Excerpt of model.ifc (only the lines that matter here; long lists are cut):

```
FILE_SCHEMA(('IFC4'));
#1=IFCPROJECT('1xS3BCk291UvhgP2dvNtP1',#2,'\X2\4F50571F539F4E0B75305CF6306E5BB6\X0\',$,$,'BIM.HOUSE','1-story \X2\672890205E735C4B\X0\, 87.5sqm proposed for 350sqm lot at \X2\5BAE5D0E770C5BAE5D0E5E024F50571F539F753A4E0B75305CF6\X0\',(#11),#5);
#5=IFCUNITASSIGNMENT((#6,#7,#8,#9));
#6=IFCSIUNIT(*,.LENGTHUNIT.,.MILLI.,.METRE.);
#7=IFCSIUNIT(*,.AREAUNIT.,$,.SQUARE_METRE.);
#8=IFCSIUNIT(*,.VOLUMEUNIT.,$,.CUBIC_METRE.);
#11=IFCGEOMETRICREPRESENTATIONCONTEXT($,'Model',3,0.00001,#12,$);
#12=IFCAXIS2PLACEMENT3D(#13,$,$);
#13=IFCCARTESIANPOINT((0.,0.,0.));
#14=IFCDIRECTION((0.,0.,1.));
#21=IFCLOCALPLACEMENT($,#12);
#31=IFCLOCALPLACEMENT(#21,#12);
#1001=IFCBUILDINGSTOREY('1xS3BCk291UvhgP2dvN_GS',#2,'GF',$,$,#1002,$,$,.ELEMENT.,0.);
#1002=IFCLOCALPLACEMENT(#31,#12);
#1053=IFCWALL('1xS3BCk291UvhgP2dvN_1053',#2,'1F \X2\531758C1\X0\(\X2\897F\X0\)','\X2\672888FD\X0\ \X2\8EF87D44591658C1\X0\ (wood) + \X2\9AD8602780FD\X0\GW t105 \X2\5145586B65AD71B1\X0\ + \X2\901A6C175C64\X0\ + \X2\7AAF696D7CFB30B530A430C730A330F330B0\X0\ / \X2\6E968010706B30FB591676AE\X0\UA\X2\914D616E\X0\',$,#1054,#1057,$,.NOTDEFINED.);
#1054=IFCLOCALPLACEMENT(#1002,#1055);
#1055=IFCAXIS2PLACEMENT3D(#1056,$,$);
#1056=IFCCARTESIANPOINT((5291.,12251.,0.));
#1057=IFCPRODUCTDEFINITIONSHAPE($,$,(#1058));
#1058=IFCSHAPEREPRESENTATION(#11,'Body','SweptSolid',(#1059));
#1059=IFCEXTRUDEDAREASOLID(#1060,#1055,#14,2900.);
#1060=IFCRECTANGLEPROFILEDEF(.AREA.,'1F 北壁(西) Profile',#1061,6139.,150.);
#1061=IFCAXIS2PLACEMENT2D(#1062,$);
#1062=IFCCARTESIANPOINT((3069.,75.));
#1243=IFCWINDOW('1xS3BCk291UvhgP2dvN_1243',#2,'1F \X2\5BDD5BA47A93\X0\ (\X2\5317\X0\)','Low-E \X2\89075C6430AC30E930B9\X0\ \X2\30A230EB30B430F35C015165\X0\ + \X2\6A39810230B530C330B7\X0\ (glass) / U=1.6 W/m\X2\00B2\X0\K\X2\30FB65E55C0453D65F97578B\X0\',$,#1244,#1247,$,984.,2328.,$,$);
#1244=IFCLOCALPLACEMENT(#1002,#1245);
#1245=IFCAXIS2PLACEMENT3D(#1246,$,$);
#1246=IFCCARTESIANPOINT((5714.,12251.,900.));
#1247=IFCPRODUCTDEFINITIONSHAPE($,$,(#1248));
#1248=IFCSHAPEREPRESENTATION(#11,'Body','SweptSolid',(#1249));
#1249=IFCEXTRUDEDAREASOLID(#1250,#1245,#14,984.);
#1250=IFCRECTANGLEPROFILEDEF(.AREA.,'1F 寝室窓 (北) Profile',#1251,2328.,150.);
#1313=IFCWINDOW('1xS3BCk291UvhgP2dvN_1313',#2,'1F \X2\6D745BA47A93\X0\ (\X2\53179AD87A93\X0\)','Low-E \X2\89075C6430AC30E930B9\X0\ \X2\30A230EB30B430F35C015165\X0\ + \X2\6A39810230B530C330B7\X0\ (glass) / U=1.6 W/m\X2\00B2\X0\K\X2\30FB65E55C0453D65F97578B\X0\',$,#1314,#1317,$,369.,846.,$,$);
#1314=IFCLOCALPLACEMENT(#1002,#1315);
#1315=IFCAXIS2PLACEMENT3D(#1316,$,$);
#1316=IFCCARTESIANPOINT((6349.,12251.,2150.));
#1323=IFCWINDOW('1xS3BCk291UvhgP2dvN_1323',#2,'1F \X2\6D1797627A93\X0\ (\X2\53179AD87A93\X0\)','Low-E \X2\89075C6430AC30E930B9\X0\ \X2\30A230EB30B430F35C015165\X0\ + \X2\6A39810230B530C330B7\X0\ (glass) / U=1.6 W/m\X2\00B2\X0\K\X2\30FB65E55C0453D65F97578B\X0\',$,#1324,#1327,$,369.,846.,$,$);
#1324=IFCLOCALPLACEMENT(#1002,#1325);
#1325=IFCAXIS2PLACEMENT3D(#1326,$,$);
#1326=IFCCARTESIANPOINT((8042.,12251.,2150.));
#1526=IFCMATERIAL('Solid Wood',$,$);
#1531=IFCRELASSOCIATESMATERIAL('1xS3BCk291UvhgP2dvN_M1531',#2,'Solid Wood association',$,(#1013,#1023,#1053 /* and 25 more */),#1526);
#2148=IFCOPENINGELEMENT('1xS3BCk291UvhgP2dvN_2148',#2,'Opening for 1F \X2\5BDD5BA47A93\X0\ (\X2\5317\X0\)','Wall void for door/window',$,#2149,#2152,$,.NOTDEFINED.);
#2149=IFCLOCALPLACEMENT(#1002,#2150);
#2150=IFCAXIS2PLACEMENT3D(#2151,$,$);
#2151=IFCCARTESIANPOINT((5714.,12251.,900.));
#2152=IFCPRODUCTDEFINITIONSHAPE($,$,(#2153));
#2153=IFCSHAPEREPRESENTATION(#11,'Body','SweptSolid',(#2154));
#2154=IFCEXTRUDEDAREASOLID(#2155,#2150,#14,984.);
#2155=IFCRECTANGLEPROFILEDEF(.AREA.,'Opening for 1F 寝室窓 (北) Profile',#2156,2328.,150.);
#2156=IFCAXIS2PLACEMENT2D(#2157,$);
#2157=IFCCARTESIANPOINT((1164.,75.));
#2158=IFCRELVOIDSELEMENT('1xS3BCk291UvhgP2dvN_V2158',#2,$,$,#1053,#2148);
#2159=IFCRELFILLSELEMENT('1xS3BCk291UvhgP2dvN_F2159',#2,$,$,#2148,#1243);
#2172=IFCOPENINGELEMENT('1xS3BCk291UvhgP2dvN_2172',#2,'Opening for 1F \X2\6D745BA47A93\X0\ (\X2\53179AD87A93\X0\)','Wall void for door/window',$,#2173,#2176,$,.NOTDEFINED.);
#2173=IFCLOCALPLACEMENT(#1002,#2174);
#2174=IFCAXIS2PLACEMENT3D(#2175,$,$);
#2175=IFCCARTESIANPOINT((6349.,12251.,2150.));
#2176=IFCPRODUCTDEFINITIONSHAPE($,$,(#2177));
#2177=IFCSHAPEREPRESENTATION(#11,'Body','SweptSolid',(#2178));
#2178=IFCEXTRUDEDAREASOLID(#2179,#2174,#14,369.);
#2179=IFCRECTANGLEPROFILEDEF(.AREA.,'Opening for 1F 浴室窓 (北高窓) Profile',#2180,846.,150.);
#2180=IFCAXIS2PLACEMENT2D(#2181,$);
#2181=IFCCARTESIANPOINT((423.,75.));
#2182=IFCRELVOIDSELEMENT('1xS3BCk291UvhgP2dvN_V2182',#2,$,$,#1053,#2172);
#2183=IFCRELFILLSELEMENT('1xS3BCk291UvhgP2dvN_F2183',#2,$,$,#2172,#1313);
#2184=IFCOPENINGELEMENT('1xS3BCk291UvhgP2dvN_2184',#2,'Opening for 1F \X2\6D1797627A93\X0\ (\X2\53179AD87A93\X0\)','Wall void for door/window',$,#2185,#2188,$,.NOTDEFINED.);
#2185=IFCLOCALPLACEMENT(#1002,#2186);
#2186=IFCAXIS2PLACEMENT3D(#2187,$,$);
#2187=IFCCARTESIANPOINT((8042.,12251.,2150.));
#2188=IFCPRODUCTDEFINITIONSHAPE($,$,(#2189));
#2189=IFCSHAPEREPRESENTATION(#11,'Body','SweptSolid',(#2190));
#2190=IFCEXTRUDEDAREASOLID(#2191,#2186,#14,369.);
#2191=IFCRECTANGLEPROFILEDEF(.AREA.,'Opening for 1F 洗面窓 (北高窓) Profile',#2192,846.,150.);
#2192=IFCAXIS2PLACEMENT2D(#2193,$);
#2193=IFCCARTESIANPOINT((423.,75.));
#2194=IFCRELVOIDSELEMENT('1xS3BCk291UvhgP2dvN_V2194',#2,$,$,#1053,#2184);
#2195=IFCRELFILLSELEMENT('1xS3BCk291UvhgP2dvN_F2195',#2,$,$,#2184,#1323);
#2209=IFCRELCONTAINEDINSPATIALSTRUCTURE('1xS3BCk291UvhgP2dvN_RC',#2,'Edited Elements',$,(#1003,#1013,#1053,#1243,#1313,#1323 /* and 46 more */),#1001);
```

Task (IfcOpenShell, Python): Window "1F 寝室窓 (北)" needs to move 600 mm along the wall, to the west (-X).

```python
import ifcopenshell
import ifcopenshell.api.geometry
import ifcopenshell.util.placement
import ifcopenshell.util.unit

model = ifcopenshell.open("model.ifc")
unit_scale = ifcopenshell.util.unit.calculate_unit_scale(model)

window = model.by_guid("1xS3BCk291UvhgP2dvN_1243")
opening = window.FillsVoids[0].RelatingOpeningElement
wall = opening.VoidsElements[0].RelatingBuildingElement

wall_matrix = ifcopenshell.util.placement.get_local_placement(wall.ObjectPlacement)
shift = wall_matrix[:3, 0] * -0.6 / unit_scale
before = ifcopenshell.util.placement.get_local_placement(window.ObjectPlacement)[:3, 3].copy()

# The window is not placed relative to its opening, so move both.
for product in (opening, window):
    matrix = ifcopenshell.util.placement.get_local_placement(product.ObjectPlacement)
    matrix[:3, 3] += shift
    ifcopenshell.api.geometry.edit_object_placement(model, product=product, matrix=matrix, is_si=False)

after = ifcopenshell.util.placement.get_local_placement(window.ObjectPlacement)[:3, 3]
print("window moved by", (after - before).round(3) + 0.0)

model.write("model_rev.ifc")
```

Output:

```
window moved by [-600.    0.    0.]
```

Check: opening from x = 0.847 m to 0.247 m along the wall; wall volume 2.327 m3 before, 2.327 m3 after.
